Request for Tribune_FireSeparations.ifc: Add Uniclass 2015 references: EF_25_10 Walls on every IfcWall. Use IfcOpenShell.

First a look at what the model holds.

```python
import ifcopenshell

model = ifcopenshell.open("Tribune_FireSeparations.ifc")
print(model.schema)
print("classifications:", [c.Name for c in model.by_type("IfcClassification")])
for ifc_class in ("IfcDoor", "IfcRoof", "IfcStair", "IfcWall", "IfcWindow"):
    print(ifc_class, len(model.by_type(ifc_class)))
```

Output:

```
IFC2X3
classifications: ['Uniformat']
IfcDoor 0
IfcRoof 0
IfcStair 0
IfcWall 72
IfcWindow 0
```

```python
import ifcopenshell
import ifcopenshell.api.classification

model = ifcopenshell.open("Tribune_FireSeparations.ifc")

# IFC2X3 requires Source and Edition and has no link from the project to the system.
system = model.create_entity("IfcClassification", Source="NBS", Edition="2015", Name="Uniclass 2015")

codes = {
    "IfcWall": ("EF_25_10", "Walls"),
}
for ifc_class, (code, name) in codes.items():
    products = model.by_type(ifc_class)
    ifcopenshell.api.classification.add_reference(
        model, products=products, classification=system, identification=code, name=name
    )
    print(code, len(products))

model.write("Tribune_FireSeparations_edited.ifc")
```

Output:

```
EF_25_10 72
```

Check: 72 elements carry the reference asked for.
